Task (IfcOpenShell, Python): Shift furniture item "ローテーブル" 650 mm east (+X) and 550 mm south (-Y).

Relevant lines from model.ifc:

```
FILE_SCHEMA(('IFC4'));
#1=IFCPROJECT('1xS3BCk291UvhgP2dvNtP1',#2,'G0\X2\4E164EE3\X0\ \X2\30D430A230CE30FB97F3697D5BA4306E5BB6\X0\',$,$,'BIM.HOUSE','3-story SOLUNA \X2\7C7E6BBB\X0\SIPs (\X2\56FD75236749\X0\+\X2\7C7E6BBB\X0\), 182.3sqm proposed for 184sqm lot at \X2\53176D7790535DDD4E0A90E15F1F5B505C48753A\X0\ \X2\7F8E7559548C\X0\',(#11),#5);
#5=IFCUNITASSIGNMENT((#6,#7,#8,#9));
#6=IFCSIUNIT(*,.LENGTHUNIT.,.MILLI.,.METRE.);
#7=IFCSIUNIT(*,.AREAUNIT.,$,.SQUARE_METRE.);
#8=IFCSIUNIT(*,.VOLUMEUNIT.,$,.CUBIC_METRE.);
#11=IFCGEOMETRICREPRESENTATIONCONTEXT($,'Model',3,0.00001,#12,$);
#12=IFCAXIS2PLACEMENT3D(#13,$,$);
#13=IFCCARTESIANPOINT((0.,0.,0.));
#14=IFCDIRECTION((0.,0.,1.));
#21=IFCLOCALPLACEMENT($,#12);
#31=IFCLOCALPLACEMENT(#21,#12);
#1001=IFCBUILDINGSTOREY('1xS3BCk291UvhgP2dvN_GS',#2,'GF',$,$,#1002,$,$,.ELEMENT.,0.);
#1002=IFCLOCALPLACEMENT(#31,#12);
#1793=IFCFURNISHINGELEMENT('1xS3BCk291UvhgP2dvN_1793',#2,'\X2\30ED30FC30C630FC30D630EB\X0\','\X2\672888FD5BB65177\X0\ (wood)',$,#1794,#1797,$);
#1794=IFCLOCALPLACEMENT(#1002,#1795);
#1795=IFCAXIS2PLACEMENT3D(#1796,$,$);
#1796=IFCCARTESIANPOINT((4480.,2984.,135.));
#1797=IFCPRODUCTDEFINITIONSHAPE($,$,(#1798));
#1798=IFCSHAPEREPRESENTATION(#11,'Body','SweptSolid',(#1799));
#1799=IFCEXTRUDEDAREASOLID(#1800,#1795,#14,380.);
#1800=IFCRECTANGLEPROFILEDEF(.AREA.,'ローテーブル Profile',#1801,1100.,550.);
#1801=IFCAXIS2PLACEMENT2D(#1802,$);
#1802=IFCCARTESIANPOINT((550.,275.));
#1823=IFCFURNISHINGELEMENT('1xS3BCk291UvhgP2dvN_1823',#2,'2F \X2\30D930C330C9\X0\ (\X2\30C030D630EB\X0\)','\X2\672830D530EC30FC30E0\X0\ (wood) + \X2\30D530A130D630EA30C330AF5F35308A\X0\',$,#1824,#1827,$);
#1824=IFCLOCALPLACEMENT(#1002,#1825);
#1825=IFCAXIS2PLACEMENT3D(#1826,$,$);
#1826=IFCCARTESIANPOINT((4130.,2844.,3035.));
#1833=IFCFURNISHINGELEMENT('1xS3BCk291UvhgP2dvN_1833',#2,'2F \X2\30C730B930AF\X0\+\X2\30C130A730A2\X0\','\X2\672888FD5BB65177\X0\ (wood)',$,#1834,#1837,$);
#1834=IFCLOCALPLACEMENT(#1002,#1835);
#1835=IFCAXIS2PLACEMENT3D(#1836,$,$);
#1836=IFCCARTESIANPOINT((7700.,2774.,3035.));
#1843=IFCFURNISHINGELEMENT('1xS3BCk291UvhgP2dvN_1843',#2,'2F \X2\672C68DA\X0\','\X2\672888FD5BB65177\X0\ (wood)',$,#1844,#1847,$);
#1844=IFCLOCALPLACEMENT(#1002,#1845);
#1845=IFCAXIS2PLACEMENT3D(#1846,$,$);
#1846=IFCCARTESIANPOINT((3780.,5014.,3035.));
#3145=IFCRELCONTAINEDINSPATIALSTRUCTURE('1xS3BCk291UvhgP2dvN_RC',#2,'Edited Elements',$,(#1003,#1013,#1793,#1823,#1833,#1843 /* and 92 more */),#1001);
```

```python
import ifcopenshell
import ifcopenshell.api.geometry
import ifcopenshell.util.placement
import ifcopenshell.util.unit

model = ifcopenshell.open("model.ifc")
unit_scale = ifcopenshell.util.unit.calculate_unit_scale(model)

item = model.by_id(1793)
matrix = ifcopenshell.util.placement.get_local_placement(item.ObjectPlacement)
matrix[0, 3] += 0.65 / unit_scale
matrix[1, 3] -= 0.55 / unit_scale
ifcopenshell.api.geometry.edit_object_placement(model, product=item, matrix=matrix, is_si=False)

print(ifcopenshell.util.placement.get_local_placement(item.ObjectPlacement).round(3) + 0.0)

model.write("model_updated.ifc")
```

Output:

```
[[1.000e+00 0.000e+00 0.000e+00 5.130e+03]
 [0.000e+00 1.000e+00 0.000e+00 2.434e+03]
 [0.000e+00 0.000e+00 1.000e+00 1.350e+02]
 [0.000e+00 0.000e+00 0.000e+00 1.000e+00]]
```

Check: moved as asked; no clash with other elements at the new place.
